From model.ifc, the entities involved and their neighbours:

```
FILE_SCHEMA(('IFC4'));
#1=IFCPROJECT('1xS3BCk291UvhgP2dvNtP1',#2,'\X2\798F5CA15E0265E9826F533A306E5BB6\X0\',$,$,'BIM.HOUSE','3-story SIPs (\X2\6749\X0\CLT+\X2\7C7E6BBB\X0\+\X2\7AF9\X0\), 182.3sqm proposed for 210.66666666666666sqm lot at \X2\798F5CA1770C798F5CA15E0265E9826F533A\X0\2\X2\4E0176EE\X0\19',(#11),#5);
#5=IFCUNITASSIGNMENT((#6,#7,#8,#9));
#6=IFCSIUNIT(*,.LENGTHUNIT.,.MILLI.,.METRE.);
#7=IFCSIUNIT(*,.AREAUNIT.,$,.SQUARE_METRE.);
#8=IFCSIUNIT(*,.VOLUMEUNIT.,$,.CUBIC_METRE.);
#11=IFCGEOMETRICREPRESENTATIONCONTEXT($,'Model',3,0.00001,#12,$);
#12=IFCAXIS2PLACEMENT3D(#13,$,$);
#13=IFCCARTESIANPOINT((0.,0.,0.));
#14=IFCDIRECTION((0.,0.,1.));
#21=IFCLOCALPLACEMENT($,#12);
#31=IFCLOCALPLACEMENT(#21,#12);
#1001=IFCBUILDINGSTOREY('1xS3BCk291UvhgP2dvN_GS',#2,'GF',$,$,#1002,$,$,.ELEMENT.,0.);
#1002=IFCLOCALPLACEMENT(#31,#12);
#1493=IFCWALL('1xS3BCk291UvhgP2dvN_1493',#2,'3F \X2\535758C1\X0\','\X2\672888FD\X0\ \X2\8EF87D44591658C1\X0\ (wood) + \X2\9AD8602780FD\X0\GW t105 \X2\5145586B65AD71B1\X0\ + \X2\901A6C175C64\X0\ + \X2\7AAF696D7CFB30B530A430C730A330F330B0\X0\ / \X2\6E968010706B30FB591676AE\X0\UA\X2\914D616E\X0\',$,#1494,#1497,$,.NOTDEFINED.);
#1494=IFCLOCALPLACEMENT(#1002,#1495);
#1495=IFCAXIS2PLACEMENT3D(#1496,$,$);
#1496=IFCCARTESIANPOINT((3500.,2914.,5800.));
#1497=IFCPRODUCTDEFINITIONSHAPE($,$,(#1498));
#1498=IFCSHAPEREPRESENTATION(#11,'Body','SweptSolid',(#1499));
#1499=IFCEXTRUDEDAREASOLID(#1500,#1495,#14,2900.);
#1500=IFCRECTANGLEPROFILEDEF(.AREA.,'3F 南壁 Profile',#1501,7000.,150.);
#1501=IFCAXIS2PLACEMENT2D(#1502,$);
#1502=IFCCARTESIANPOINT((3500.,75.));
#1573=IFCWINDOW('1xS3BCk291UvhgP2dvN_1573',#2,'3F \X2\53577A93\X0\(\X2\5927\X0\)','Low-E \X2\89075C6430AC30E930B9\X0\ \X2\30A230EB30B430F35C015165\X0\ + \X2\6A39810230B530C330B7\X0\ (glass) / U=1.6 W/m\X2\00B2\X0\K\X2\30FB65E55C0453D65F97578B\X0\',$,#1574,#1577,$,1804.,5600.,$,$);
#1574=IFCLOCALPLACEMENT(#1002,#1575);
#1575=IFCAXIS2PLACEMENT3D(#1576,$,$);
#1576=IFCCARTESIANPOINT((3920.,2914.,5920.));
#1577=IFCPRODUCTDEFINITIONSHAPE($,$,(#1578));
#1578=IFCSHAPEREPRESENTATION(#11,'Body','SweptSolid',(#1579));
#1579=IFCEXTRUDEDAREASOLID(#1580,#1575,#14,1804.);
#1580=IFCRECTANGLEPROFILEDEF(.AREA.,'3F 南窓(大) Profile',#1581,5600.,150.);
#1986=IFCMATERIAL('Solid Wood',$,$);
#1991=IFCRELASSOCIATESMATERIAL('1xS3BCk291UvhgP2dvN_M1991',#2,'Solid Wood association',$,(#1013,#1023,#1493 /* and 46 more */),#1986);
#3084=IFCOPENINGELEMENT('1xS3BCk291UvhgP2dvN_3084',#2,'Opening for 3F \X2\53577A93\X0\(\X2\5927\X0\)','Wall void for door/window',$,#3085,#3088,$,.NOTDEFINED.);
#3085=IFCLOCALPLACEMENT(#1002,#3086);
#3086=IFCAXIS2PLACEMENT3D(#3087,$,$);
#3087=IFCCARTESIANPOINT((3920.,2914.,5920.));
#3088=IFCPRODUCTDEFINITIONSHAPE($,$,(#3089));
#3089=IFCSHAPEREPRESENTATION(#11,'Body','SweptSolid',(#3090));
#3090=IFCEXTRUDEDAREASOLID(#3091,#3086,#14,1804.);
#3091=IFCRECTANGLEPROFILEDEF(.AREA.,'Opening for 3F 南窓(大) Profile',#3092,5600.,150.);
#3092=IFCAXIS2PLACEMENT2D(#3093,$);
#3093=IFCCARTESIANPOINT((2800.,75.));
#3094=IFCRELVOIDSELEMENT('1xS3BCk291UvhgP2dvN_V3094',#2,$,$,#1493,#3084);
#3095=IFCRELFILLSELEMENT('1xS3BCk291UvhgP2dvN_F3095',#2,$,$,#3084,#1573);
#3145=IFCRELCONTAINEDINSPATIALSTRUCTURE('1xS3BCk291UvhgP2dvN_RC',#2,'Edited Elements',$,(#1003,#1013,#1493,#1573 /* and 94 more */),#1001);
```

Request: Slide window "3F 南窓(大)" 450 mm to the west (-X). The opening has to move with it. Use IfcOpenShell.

```python
import ifcopenshell
import ifcopenshell.api.geometry
import ifcopenshell.util.placement

model = ifcopenshell.open("model.ifc")

window = model.by_guid("1xS3BCk291UvhgP2dvN_1573")
opening = window.FillsVoids[0].RelatingOpeningElement
wall = opening.VoidsElements[0].RelatingBuildingElement

wall_matrix = ifcopenshell.util.placement.get_local_placement(wall.ObjectPlacement)
shift = wall_matrix[:3, 0] * -450.0
before = ifcopenshell.util.placement.get_local_placement(window.ObjectPlacement)[:3, 3].copy()

# The window is not placed relative to its opening, so move both.
for product in (opening, window):
    matrix = ifcopenshell.util.placement.get_local_placement(product.ObjectPlacement)
    matrix[:3, 3] += shift
    ifcopenshell.api.geometry.edit_object_placement(model, product=product, matrix=matrix, is_si=False)

after = ifcopenshell.util.placement.get_local_placement(window.ObjectPlacement)[:3, 3]
print("window moved by", (after - before).round(3) + 0.0)

model.write("model-out.ifc")
```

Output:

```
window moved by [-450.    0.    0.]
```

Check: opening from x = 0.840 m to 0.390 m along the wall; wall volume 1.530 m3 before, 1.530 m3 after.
